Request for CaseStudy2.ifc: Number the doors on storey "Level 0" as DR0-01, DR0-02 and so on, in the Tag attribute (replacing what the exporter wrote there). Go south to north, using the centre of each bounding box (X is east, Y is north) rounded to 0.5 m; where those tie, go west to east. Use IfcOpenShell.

First a look at what the model holds.

```python
import ifcopenshell
import ifcopenshell.util.element
import ifcopenshell.util.placement

model = ifcopenshell.open("CaseStudy2.ifc")
print(model.schema)
storey = next(s for s in model.by_type("IfcBuildingStorey") if s.Name == "Level 0")
doors = [e for e in ifcopenshell.util.element.get_decomposition(storey) if e.is_a("IfcDoor")]
for e in sorted(doors, key=lambda e: e.id()):
    origin = ifcopenshell.util.placement.get_local_placement(e.ObjectPlacement)[:3, 3]
    print(e.id(), e.Tag, e.Name, origin.round(2) + 0.0, sep=" | ")
```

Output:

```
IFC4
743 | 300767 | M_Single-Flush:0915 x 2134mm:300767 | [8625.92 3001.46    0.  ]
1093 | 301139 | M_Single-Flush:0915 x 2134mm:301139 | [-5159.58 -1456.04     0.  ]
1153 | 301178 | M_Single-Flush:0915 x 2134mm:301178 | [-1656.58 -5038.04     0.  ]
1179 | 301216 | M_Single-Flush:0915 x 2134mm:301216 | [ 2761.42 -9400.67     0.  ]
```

```python
import ifcopenshell
import ifcopenshell.geom
import ifcopenshell.util.element
import ifcopenshell.util.shape

model = ifcopenshell.open("CaseStudy2.ifc")
settings = ifcopenshell.geom.settings()
settings.set("use-world-coords", True)


def centre(element):
    shape = ifcopenshell.geom.create_shape(settings, element)
    return ifcopenshell.util.shape.get_bbox_centroid(shape.geometry)


storey = next(s for s in model.by_type("IfcBuildingStorey") if s.Name == "Level 0")
doors = [e for e in ifcopenshell.util.element.get_decomposition(storey) if e.is_a("IfcDoor")]

# Insertion points can sit at a corner or the storey origin, so sort by the geometry (in metres).
centres = {e: centre(e) for e in doors}
doors.sort(key=lambda e: (round(centres[e][1] / 0.5), centres[e][0]))

for i, e in enumerate(doors, start=1):
    number = f"DR0-{i:02d}"
    e.Tag = number
    print(e.id(), number)

model.write("CaseStudy2_updated.ifc")
```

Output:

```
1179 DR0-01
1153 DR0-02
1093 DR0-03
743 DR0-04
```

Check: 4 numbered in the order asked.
